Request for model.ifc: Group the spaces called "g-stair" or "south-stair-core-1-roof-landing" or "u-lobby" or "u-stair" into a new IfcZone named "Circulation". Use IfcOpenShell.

First a look at what the model holds.

```python
import ifcopenshell

model = ifcopenshell.open("model.ifc")
print(model.schema)
seen = {}
for space in model.by_type("IfcSpace"):
    seen[space.LongName] = seen.get(space.LongName, 0) + 1
for name, count in sorted(seen.items(), key=str):
    print(count, "x", name)
print("zones:", [z.Name for z in model.by_type("IfcZone")][:20])
```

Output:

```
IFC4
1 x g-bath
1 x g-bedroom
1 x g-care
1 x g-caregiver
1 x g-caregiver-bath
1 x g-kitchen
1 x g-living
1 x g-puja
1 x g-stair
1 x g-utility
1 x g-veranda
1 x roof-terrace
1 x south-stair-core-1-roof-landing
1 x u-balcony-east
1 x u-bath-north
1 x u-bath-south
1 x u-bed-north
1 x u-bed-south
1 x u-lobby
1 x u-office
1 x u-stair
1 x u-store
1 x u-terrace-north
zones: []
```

```python
import ifcopenshell
import ifcopenshell.api.group
import ifcopenshell.api.root

model = ifcopenshell.open("model.ifc")

names = {"g-stair", "south-stair-core-1-roof-landing", "u-lobby", "u-stair"}
spaces = [s for s in model.by_type("IfcSpace") if s.LongName in names]

zone = ifcopenshell.api.root.create_entity(model, ifc_class="IfcZone", name="Circulation")
ifcopenshell.api.group.assign_group(model, products=spaces, group=zone)
print(len(spaces), "spaces in", zone.Name)

model.write("model_edited.ifc")
```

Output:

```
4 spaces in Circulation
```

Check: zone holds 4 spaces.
